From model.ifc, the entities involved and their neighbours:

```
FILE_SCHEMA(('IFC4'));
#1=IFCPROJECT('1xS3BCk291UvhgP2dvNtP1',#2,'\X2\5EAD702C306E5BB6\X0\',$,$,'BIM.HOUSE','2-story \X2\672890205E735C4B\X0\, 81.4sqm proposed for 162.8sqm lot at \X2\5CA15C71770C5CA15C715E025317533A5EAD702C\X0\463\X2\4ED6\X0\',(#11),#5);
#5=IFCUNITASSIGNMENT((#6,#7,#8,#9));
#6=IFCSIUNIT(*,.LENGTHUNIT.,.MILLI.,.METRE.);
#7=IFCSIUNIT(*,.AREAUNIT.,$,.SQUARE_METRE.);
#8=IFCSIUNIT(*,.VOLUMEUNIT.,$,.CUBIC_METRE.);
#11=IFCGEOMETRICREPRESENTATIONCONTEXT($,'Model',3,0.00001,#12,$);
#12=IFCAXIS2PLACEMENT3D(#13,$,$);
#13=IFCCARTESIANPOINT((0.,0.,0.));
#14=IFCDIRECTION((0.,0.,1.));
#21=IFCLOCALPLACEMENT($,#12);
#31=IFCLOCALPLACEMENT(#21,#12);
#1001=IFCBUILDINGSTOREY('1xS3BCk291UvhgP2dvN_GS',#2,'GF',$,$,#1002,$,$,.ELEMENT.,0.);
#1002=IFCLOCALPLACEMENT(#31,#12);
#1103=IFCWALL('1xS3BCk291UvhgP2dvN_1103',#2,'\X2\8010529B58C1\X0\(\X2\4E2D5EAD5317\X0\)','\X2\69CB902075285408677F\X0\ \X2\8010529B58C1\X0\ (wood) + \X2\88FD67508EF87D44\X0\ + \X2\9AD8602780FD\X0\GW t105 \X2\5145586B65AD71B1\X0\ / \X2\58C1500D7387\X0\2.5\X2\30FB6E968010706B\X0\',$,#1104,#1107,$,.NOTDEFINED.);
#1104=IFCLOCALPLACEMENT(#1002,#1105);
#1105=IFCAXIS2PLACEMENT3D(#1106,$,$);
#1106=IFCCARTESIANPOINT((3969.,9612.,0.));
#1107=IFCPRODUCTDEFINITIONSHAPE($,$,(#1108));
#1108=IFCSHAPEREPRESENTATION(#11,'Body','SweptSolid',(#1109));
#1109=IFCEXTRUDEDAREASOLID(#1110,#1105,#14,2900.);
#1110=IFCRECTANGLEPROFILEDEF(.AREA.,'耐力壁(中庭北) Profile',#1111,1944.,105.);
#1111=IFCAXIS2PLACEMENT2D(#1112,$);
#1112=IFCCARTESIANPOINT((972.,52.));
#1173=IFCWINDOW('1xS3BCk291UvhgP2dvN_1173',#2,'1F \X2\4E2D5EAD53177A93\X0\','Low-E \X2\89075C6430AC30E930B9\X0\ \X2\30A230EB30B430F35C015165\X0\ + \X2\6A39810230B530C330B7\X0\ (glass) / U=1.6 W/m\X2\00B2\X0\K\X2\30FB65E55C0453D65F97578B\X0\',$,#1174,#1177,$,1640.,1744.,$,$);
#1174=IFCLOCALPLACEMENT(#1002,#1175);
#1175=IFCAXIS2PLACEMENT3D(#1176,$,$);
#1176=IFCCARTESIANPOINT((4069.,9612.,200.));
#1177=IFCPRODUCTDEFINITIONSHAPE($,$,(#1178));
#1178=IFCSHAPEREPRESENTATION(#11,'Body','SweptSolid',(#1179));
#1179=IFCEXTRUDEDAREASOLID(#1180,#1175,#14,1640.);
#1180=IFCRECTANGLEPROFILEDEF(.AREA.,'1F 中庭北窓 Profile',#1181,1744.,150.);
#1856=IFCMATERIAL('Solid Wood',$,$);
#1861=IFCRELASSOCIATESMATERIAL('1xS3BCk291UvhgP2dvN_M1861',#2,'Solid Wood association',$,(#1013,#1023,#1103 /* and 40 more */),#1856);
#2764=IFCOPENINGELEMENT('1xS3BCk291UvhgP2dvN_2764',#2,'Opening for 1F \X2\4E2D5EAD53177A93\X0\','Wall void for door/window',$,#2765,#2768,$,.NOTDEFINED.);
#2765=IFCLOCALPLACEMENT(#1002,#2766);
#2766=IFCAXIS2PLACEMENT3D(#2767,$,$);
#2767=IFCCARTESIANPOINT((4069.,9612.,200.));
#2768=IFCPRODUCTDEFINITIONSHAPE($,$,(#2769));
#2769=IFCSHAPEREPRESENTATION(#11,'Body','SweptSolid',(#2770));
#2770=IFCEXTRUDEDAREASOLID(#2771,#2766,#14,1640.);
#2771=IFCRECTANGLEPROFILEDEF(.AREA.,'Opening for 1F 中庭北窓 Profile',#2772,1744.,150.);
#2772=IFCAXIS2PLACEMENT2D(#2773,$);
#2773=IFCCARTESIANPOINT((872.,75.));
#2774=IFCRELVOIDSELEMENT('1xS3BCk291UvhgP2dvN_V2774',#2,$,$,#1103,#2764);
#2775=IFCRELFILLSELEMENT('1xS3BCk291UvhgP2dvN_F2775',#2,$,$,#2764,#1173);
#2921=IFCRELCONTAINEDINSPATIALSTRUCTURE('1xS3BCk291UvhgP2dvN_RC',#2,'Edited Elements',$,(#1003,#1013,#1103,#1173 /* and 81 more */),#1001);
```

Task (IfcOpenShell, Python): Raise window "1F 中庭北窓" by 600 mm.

```python
import numpy as np
import ifcopenshell
import ifcopenshell.api.geometry
import ifcopenshell.util.placement
import ifcopenshell.util.unit

model = ifcopenshell.open("model.ifc")
unit_scale = ifcopenshell.util.unit.calculate_unit_scale(model)

window = model.by_guid("1xS3BCk291UvhgP2dvN_1173")
opening = window.FillsVoids[0].RelatingOpeningElement
dz = 0.6 / unit_scale

shift = np.array([0.0, 0.0, dz])
# The window is not placed relative to its opening, so move both.
for product in (opening, window):
    matrix = ifcopenshell.util.placement.get_local_placement(product.ObjectPlacement)
    matrix[:3, 3] += shift
    ifcopenshell.api.geometry.edit_object_placement(model, product=product, matrix=matrix, is_si=False)

print(f"moved by {dz * unit_scale:+.3f} m")

model.write("model_v2.ifc")
```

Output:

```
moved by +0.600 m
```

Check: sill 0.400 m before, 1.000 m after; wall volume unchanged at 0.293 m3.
